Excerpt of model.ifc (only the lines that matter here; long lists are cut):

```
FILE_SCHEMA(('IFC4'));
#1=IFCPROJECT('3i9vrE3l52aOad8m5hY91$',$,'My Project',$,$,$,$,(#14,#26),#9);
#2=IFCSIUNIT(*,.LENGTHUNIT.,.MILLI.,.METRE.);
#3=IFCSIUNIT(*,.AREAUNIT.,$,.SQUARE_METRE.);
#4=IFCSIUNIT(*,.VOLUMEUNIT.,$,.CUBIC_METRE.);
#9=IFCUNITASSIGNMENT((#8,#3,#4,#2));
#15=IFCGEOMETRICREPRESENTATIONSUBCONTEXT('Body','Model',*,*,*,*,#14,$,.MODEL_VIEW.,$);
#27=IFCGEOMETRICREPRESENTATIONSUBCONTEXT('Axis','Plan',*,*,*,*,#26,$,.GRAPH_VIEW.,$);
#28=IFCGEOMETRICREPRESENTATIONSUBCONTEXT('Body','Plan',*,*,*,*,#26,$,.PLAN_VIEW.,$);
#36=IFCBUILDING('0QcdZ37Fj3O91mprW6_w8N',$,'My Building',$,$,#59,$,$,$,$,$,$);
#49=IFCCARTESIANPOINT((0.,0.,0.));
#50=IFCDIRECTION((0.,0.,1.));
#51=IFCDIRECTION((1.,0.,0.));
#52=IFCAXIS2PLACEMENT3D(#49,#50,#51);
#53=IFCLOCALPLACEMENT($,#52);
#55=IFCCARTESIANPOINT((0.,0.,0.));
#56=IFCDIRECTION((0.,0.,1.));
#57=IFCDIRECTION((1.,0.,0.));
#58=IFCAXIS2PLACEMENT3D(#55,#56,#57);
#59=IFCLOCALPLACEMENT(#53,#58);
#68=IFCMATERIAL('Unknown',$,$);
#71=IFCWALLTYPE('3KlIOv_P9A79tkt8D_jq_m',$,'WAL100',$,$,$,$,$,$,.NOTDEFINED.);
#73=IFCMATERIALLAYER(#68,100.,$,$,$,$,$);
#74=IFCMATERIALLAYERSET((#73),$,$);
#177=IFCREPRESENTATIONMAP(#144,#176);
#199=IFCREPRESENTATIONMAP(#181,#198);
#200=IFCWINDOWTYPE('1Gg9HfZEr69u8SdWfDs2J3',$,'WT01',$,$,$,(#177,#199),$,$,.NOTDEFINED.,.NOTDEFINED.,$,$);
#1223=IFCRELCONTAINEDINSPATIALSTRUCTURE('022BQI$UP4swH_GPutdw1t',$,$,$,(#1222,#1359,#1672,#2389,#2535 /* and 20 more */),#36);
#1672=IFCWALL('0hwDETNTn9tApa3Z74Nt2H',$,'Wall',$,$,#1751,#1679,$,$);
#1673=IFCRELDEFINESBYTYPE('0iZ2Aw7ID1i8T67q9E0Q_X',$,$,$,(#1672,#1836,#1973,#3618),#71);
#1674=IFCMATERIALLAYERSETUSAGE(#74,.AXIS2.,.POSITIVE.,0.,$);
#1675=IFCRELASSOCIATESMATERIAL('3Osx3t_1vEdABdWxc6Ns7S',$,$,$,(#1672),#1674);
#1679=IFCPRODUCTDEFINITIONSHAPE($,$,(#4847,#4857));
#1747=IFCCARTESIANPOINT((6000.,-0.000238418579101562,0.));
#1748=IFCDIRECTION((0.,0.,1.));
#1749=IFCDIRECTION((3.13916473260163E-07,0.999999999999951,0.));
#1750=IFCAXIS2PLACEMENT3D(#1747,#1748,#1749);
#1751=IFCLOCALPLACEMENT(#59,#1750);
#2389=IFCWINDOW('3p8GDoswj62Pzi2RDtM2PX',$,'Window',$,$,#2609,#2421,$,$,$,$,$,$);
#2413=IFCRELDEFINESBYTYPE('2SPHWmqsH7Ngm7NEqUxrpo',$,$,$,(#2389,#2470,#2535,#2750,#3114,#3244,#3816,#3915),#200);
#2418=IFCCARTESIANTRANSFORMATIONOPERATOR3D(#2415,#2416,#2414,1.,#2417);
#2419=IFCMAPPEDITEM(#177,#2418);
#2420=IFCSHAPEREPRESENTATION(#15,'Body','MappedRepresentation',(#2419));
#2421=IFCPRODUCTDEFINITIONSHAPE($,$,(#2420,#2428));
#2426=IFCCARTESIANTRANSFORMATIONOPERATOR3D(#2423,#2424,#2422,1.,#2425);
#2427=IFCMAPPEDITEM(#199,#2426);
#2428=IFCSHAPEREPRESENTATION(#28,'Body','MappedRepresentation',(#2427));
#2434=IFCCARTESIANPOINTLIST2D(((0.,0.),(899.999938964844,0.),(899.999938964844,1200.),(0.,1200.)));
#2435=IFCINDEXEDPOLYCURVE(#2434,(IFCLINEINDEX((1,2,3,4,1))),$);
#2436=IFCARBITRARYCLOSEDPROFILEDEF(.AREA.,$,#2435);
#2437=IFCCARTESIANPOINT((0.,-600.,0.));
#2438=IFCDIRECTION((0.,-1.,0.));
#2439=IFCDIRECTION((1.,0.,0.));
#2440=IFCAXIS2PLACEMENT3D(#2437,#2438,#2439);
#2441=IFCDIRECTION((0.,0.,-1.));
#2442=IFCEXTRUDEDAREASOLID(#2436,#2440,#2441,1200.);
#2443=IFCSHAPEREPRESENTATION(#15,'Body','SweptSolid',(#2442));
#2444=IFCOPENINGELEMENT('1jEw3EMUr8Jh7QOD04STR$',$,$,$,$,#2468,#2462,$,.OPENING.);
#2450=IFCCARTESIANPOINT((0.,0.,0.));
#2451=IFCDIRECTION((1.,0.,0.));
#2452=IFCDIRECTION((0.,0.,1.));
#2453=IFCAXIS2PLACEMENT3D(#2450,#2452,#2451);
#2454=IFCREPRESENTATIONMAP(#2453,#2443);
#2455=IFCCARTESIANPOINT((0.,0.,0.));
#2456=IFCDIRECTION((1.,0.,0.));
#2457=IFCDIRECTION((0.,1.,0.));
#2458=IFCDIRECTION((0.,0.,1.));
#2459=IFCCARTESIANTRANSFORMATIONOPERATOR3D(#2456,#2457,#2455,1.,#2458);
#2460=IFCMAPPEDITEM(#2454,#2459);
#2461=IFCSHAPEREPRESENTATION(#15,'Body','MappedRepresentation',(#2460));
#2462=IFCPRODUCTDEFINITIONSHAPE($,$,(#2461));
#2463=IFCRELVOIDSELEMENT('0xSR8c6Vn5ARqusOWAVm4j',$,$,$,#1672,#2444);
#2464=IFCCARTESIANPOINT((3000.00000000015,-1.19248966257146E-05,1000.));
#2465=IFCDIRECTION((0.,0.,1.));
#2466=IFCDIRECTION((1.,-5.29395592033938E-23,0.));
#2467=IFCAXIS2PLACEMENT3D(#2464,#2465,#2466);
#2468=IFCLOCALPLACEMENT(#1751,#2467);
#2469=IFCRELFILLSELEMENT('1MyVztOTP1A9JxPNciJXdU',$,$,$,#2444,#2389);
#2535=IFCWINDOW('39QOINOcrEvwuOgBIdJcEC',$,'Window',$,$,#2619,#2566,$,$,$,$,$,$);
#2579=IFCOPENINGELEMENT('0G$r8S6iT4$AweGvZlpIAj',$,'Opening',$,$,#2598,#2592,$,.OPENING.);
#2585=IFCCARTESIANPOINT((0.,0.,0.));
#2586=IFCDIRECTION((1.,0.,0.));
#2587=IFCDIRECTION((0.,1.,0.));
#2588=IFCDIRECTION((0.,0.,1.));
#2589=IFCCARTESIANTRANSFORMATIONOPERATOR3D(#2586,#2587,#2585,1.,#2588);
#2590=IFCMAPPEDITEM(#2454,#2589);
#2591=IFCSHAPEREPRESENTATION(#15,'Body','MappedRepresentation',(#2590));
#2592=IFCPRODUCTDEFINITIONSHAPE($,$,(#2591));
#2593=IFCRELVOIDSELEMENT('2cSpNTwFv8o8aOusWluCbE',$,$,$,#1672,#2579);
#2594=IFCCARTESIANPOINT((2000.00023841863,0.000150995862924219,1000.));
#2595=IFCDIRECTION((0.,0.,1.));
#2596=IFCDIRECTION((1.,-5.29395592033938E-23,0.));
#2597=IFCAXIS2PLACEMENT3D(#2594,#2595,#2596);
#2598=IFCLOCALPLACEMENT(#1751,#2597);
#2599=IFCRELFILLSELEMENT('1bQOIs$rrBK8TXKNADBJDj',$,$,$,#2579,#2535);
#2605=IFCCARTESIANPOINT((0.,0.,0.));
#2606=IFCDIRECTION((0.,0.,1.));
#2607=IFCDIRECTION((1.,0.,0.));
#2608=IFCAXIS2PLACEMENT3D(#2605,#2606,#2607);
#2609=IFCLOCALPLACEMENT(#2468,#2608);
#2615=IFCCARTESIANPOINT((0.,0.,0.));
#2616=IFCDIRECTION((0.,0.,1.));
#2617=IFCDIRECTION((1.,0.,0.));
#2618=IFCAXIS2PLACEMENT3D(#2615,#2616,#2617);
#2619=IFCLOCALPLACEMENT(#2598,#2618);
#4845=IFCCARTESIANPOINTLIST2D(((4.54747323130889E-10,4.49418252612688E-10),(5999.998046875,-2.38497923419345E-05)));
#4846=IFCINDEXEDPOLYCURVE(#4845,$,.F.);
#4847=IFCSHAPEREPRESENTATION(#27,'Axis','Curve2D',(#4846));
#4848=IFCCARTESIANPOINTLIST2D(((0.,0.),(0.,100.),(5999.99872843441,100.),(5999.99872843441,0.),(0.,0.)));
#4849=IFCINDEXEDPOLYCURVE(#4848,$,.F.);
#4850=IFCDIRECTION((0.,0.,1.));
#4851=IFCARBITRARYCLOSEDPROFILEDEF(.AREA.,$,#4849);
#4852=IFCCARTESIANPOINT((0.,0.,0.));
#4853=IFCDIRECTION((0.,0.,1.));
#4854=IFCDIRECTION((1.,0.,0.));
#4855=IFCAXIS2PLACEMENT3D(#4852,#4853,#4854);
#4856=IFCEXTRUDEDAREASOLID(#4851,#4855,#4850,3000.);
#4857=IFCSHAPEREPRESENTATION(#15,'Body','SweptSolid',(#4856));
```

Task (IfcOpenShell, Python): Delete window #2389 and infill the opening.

```python
import ifcopenshell
import ifcopenshell.api.feature
import ifcopenshell.api.root
import ifcopenshell.geom
import ifcopenshell.util.shape

model = ifcopenshell.open("model.ifc")
settings = ifcopenshell.geom.settings()


def volume(element):
    """Net volume in cubic metres, openings subtracted."""
    shape = ifcopenshell.geom.create_shape(settings, element)
    return ifcopenshell.util.shape.get_volume(shape.geometry)


window = model.by_id(2389)
opening = window.FillsVoids[0].RelatingOpeningElement
wall = opening.VoidsElements[0].RelatingBuildingElement
before = volume(wall)

ifcopenshell.api.root.remove_product(model, product=window)
ifcopenshell.api.feature.remove_feature(model, feature=opening)

after = volume(wall)

print(f"wall volume {before:.3f} -> {after:.3f} m3")

model.write("model_rev.ifc")
```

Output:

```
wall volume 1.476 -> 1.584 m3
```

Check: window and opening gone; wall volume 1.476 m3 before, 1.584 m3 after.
